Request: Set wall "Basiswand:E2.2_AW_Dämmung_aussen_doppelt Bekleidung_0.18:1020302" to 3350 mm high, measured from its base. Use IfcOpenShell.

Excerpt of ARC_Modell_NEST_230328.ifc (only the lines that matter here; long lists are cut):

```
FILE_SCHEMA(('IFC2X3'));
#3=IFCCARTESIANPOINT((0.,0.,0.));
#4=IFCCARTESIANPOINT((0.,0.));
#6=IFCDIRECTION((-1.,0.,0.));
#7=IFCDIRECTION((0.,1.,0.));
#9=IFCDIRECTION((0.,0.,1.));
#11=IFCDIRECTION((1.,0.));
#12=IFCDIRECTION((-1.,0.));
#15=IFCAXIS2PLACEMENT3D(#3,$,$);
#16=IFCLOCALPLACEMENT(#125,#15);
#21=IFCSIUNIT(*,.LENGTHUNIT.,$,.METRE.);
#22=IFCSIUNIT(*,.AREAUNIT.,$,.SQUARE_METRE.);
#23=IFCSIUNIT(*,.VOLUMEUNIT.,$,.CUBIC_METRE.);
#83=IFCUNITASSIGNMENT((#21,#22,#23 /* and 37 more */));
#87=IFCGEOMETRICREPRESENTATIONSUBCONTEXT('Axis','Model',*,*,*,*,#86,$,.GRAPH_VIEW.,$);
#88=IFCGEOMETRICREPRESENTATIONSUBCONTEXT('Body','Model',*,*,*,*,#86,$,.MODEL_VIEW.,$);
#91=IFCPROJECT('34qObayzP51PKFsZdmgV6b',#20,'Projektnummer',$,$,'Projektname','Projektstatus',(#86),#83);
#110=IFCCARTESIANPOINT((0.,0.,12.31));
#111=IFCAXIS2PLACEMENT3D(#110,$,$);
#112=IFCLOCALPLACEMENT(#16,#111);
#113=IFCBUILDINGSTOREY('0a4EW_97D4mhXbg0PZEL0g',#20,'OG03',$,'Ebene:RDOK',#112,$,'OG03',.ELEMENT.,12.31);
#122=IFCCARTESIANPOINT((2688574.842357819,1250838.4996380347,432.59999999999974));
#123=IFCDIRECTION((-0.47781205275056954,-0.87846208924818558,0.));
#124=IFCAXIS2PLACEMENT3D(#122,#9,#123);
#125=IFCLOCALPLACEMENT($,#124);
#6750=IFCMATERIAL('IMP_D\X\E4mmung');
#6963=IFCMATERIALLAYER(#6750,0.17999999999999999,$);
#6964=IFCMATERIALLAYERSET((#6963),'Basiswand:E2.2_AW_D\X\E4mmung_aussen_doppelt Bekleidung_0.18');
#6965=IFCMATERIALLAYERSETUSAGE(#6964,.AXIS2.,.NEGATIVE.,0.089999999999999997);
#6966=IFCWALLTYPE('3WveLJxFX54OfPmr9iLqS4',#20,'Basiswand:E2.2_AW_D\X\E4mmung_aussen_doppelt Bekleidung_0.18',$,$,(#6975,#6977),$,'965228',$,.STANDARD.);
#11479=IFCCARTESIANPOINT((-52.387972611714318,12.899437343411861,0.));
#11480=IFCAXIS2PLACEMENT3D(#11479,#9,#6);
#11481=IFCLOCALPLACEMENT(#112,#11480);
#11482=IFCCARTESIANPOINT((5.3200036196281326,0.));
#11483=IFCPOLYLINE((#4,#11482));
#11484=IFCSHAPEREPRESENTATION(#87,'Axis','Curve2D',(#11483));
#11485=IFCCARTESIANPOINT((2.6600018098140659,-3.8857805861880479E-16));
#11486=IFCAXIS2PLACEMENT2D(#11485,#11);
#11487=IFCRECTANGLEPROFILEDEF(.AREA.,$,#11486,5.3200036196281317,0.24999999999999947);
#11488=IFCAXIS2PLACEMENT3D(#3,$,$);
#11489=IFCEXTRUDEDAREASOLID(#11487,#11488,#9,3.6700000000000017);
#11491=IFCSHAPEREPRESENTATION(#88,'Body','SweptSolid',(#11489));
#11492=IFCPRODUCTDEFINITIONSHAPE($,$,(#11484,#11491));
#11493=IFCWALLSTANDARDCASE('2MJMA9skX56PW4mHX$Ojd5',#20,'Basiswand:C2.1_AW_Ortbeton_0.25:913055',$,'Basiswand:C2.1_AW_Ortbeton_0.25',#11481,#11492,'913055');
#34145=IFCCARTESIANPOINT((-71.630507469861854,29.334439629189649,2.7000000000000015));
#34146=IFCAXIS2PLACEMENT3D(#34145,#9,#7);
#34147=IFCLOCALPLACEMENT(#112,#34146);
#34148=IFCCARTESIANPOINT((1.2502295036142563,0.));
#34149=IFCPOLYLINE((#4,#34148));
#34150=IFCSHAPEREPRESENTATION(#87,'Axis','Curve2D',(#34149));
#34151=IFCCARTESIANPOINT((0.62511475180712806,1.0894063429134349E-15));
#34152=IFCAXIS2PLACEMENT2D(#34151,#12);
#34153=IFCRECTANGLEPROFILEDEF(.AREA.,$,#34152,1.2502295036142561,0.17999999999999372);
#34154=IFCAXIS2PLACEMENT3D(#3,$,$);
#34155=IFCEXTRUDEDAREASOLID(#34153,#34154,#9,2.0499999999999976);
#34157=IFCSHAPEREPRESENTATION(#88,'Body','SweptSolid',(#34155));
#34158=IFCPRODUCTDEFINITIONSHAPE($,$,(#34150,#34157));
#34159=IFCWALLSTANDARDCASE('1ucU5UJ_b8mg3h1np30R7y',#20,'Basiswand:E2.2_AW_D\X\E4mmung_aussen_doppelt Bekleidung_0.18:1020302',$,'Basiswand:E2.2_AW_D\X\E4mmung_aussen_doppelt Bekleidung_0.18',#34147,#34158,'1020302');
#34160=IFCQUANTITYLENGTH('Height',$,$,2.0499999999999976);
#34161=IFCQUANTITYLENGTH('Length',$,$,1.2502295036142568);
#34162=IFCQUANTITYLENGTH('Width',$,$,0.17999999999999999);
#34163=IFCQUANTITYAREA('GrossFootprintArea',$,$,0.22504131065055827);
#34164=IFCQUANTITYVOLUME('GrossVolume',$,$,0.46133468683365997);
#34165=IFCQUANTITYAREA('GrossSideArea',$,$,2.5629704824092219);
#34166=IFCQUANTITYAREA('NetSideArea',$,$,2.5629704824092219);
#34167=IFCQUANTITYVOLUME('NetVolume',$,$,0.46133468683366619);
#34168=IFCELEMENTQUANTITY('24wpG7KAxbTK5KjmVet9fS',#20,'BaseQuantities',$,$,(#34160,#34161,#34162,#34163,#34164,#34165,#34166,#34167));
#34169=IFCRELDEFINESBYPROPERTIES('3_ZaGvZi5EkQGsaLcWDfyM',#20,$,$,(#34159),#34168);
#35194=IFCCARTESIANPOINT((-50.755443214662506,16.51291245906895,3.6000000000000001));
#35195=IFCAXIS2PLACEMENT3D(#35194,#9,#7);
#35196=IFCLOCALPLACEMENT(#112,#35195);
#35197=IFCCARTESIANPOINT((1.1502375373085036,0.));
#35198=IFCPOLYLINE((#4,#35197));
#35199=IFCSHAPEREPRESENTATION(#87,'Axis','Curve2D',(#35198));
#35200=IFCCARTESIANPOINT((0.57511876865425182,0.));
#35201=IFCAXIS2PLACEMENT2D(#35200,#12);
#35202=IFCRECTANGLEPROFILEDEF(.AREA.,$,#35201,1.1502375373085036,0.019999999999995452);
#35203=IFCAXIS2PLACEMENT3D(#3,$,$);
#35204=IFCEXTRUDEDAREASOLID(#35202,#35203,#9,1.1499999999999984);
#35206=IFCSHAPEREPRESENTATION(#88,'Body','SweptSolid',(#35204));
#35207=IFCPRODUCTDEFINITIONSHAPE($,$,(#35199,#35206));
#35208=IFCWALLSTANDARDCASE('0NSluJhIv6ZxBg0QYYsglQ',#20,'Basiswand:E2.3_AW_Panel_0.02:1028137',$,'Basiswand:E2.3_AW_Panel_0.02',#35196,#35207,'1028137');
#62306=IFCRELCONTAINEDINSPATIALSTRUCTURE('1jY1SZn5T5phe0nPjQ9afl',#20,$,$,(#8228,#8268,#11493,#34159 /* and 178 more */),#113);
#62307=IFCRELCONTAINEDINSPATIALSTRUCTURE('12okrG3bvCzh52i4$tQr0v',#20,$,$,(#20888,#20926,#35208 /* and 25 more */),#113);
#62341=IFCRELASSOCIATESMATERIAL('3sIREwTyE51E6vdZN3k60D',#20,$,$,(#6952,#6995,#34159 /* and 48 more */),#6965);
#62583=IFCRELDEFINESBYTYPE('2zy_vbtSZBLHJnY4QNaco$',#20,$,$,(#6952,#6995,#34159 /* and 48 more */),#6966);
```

```python
import ifcopenshell
import ifcopenshell.api.pset
import ifcopenshell.geom
import ifcopenshell.util.element
import ifcopenshell.util.representation
import ifcopenshell.util.shape
import ifcopenshell.util.unit

model = ifcopenshell.open("ARC_Modell_NEST_230328.ifc")
unit_scale = ifcopenshell.util.unit.calculate_unit_scale(model)
area_scale = ifcopenshell.util.unit.calculate_unit_scale(model, "AREAUNIT")
volume_scale = ifcopenshell.util.unit.calculate_unit_scale(model, "VOLUMEUNIT")
settings = ifcopenshell.geom.settings()


def volume(element):
    """Net volume in cubic metres, openings subtracted."""
    shape = ifcopenshell.geom.create_shape(settings, element)
    return ifcopenshell.util.shape.get_volume(shape.geometry)


wall = model.by_id(34159)
before = volume(wall)

body = ifcopenshell.util.representation.get_representation(wall, "Model", "Body")
solid = body.Items[0]
old_height = solid.Depth
solid.Depth = 3.35
after = volume(wall)
thickness = 0.18  # wall thickness in metres

# Update the stored height, areas and volumes.
qto = model.by_id(ifcopenshell.util.element.get_pset(wall, "BaseQuantities", should_inherit=False)["id"])
ifcopenshell.api.pset.edit_qto(model, qto=qto, properties={
    "Height": solid.Depth,
    "GrossVolume": ifcopenshell.util.element.get_pset(wall, "BaseQuantities", "GrossVolume") * solid.Depth / old_height,
    "GrossSideArea": ifcopenshell.util.element.get_pset(wall, "BaseQuantities", "GrossSideArea") * solid.Depth / old_height,
    "NetSideArea": after / thickness / area_scale,
    "NetVolume": after / volume_scale,
})

print(f"height {old_height:g} -> {solid.Depth:g}, volume {before:.3f} -> {after:.3f} m3")

model.write("ARC_Modell_NEST_230328_rev.ifc")
```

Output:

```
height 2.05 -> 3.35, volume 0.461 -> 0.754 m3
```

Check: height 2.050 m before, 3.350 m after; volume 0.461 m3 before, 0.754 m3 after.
